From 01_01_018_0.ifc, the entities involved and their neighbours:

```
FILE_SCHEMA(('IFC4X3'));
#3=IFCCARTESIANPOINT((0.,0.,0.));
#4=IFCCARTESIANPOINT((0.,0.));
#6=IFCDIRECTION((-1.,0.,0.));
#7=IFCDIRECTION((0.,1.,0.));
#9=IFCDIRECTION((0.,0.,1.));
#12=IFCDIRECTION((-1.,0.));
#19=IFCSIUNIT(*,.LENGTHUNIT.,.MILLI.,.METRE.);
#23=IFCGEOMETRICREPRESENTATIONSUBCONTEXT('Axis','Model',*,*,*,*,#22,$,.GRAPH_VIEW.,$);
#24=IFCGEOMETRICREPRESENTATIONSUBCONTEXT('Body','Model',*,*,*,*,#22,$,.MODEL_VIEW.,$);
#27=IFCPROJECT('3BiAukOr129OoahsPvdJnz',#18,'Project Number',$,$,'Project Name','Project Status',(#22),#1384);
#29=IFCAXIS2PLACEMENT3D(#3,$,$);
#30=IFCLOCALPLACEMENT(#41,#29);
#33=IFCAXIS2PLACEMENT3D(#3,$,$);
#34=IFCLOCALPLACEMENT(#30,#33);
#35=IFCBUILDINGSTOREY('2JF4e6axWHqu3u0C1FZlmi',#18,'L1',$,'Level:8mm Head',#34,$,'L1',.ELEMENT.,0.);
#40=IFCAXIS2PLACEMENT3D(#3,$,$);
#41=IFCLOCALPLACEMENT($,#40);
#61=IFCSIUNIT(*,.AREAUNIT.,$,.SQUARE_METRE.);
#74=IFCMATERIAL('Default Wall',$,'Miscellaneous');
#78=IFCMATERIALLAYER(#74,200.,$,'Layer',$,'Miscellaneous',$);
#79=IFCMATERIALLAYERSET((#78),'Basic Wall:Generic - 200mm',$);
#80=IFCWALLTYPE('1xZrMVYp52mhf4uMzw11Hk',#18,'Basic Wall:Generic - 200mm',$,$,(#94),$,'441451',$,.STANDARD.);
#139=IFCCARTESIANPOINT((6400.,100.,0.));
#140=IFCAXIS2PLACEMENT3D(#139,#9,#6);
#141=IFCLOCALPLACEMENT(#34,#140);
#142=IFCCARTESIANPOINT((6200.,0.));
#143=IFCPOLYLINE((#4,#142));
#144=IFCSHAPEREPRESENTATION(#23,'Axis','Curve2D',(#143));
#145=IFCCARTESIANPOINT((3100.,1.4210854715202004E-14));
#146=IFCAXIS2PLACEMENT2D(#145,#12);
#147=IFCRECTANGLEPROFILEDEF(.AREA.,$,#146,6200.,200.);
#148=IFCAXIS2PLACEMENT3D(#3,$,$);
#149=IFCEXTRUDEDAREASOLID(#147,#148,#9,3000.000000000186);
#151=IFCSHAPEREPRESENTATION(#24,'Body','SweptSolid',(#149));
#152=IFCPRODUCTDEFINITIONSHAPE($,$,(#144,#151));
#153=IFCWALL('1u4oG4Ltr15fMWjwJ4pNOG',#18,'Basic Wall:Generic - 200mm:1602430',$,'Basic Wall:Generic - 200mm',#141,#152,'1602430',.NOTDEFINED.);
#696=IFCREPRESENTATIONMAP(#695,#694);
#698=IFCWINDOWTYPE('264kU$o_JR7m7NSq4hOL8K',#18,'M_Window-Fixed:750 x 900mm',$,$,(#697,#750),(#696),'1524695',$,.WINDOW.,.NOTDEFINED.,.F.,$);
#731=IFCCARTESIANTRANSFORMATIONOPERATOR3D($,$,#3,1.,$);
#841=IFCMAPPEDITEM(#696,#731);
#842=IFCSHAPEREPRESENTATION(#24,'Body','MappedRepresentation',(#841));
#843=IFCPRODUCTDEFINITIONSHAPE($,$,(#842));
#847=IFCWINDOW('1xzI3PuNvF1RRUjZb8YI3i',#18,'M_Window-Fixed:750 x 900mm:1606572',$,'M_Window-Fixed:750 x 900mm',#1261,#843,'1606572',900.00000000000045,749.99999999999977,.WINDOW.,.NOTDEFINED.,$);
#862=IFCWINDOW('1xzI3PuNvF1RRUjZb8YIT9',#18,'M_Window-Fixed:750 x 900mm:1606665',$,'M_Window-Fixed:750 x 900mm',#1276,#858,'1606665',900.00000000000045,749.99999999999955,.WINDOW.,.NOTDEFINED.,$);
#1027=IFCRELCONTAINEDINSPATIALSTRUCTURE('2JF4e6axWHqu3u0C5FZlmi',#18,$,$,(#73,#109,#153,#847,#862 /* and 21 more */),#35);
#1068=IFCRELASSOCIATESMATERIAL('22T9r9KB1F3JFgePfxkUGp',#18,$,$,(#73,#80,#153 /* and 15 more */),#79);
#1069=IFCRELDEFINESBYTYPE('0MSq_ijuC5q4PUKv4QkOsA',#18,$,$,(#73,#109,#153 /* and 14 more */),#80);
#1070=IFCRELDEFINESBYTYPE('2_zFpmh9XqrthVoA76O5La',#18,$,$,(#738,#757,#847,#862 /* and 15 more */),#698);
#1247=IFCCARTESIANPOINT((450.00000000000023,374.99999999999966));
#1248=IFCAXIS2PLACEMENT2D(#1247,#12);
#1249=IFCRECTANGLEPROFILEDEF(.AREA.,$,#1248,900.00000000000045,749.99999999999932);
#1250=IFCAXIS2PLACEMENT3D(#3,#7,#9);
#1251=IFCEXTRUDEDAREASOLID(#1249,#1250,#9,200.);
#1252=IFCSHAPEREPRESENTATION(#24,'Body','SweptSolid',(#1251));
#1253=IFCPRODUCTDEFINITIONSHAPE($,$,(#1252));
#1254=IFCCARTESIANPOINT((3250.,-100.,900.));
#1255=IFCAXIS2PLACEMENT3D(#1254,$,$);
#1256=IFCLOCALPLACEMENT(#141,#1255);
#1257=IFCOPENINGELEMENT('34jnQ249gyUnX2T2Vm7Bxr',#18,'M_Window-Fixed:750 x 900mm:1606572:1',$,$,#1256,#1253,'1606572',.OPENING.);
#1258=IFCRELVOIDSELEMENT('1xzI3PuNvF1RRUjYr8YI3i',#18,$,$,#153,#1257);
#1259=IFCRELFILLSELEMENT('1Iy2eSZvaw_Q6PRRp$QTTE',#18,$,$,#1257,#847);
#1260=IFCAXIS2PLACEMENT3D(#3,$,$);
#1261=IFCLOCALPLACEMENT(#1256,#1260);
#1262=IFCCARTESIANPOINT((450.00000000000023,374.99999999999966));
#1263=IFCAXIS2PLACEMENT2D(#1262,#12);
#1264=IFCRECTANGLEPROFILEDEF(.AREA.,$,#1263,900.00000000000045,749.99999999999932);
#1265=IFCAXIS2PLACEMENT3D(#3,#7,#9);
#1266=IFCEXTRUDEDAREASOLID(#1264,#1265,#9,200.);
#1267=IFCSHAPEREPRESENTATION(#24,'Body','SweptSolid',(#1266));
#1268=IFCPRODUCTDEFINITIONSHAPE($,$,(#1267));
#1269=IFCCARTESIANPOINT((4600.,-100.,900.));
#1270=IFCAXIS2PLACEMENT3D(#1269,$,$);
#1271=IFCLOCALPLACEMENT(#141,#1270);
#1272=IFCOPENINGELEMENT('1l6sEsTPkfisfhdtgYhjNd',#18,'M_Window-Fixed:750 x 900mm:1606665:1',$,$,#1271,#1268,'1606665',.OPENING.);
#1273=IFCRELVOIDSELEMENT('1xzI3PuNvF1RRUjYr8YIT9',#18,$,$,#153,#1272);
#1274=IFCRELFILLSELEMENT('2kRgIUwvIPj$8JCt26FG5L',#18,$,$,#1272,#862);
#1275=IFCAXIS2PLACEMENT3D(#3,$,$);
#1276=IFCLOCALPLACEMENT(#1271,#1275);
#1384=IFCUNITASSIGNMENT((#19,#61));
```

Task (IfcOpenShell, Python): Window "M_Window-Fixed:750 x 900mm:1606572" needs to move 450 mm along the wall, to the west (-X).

```python
import ifcopenshell
import ifcopenshell.api.geometry
import ifcopenshell.util.placement

model = ifcopenshell.open("01_01_018_0.ifc")

window = model.by_id(847)
opening = window.FillsVoids[0].RelatingOpeningElement
wall = opening.VoidsElements[0].RelatingBuildingElement

wall_matrix = ifcopenshell.util.placement.get_local_placement(wall.ObjectPlacement)
shift = wall_matrix[:3, 0] * 450.0
before = ifcopenshell.util.placement.get_local_placement(window.ObjectPlacement)[:3, 3].copy()

# The window is placed relative to its opening, so it follows when the opening moves.
matrix = ifcopenshell.util.placement.get_local_placement(opening.ObjectPlacement)
matrix[:3, 3] += shift
ifcopenshell.api.geometry.edit_object_placement(
    model, product=opening, matrix=matrix, is_si=False, should_transform_children=True
)

after = ifcopenshell.util.placement.get_local_placement(window.ObjectPlacement)[:3, 3]
print("window moved by", (after - before).round(3) + 0.0)

model.write("01_01_018_0_rev.ifc")
```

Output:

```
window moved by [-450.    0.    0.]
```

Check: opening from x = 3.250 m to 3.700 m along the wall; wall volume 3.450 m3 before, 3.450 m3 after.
